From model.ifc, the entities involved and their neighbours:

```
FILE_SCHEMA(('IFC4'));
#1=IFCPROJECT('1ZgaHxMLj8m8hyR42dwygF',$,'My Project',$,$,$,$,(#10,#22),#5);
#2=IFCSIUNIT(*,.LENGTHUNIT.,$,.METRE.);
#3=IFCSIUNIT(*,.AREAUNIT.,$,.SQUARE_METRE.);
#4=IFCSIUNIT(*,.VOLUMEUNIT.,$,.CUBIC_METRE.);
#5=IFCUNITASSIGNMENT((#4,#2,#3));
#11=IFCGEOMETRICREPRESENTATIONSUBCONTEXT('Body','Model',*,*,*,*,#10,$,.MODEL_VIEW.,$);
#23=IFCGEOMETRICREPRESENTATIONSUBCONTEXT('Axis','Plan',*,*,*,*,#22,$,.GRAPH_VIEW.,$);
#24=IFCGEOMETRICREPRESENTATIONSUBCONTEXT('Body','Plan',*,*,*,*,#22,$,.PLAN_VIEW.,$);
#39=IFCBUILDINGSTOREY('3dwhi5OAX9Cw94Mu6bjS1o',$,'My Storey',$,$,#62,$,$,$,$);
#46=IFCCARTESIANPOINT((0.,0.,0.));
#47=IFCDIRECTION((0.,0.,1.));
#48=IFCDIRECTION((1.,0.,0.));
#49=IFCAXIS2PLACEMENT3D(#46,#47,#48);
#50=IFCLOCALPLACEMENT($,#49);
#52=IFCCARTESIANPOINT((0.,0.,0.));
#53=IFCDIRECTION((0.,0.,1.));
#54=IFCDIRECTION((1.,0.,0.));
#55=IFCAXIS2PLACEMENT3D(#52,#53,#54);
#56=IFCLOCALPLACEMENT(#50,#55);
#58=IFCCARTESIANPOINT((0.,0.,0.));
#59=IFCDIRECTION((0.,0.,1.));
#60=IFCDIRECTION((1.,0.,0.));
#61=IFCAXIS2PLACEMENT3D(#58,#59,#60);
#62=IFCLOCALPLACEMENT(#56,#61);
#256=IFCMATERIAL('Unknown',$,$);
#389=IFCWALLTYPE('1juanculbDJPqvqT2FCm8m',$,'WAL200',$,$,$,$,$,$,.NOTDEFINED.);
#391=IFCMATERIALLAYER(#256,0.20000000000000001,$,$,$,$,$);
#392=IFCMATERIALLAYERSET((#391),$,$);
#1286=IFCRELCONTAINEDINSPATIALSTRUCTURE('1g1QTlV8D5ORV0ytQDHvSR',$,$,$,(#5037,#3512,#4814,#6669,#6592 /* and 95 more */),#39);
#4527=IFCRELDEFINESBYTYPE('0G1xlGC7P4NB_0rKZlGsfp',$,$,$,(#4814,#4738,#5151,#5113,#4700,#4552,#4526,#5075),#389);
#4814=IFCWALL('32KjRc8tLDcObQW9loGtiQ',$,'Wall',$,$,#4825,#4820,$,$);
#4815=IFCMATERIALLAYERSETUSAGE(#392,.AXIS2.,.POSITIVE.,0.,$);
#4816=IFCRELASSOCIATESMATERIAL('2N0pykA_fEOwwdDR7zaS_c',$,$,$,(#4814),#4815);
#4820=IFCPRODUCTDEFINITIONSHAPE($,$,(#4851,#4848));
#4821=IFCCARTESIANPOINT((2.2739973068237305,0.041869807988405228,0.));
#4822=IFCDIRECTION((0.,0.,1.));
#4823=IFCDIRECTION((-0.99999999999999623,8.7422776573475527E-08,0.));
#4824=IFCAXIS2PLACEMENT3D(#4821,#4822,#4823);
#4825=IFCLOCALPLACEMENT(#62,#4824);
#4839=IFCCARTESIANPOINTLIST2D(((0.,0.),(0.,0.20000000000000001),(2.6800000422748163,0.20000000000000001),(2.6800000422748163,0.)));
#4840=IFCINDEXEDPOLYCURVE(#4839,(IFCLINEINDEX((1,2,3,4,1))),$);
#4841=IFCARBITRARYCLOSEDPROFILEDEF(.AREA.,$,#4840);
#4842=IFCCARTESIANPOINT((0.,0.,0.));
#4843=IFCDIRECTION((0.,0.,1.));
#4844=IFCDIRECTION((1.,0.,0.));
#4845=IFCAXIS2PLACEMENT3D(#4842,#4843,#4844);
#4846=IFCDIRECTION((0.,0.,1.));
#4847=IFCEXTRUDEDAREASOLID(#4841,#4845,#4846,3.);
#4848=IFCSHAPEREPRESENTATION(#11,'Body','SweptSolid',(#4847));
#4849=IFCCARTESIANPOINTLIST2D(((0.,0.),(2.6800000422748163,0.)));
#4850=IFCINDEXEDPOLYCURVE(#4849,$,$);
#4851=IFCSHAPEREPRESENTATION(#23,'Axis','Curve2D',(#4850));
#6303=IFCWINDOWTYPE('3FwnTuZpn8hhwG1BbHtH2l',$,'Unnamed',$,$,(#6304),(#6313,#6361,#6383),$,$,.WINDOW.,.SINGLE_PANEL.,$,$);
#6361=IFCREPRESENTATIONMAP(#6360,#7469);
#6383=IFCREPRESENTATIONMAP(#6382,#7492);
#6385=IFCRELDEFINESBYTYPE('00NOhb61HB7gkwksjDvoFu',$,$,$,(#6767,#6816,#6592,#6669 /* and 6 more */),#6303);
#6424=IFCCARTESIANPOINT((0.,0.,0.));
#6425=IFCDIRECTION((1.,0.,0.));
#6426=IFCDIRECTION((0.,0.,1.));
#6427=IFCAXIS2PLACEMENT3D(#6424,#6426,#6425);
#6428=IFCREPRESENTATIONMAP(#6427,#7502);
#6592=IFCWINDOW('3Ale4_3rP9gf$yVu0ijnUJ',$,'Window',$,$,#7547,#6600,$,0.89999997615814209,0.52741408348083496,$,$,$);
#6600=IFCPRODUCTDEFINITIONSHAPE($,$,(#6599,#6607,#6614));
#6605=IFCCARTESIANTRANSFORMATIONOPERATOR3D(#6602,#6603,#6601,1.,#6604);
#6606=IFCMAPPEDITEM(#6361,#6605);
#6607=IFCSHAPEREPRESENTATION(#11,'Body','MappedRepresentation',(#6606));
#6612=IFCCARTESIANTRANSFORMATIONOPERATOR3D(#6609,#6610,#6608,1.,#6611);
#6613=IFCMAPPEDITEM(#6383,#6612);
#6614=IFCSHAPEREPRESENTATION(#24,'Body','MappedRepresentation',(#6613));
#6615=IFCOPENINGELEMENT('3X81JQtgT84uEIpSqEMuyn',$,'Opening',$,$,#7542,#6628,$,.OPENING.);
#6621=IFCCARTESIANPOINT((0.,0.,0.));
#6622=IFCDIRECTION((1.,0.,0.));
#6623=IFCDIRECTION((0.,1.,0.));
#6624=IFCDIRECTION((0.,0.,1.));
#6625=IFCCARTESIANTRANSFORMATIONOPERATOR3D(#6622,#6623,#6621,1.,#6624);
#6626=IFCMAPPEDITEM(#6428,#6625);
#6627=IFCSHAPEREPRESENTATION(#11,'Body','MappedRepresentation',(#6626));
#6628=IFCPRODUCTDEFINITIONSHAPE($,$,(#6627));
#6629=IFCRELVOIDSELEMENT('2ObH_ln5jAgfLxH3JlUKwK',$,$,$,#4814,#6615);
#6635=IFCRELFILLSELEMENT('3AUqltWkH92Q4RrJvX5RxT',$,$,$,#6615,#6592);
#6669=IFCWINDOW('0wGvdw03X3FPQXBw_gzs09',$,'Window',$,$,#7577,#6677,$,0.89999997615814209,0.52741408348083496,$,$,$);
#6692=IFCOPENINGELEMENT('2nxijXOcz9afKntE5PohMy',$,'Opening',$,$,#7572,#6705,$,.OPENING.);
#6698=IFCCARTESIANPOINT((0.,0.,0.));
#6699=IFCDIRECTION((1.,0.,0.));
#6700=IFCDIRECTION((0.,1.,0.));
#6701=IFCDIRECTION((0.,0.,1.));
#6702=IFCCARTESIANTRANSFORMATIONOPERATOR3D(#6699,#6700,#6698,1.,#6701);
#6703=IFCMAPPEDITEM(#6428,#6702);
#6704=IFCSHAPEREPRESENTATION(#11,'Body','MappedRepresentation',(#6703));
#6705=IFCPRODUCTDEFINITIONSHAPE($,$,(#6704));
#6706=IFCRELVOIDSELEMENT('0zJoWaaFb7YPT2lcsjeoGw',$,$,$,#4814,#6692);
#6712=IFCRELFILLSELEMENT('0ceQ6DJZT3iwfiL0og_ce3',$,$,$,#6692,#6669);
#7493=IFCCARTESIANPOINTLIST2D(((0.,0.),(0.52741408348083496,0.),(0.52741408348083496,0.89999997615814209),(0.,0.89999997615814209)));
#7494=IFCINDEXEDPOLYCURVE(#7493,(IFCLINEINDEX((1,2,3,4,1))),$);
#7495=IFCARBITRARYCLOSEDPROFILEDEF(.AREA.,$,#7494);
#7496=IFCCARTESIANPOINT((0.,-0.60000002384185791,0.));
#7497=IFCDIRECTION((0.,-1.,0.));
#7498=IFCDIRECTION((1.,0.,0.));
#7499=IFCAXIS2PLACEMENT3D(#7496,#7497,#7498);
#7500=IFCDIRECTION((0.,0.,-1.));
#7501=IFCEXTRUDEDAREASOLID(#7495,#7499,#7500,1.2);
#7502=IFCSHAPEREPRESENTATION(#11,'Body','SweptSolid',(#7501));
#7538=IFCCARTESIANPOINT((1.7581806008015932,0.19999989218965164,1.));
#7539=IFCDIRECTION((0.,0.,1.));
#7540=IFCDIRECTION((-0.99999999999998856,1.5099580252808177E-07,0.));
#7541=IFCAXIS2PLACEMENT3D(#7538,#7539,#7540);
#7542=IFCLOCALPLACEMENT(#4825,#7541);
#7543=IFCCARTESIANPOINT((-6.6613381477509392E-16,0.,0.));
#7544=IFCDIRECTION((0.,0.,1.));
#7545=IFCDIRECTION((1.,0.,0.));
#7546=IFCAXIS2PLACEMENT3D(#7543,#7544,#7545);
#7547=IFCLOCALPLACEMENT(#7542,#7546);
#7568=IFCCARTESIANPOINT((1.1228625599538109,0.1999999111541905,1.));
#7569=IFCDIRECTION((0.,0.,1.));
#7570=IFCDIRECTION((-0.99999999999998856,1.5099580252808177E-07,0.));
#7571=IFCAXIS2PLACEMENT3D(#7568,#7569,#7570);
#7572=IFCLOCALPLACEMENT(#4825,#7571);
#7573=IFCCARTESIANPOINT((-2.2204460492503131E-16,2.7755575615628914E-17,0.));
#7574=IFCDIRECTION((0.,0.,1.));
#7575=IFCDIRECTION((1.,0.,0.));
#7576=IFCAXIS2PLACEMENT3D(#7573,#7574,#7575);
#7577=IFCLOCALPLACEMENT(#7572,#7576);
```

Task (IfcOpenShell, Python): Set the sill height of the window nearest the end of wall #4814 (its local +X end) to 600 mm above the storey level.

```python
import numpy as np
import ifcopenshell
import ifcopenshell.api.geometry
import ifcopenshell.geom
import ifcopenshell.util.element
import ifcopenshell.util.placement
import ifcopenshell.util.shape
import ifcopenshell.util.unit

model = ifcopenshell.open("model.ifc")
unit_scale = ifcopenshell.util.unit.calculate_unit_scale(model)

window = model.by_id(6592)
opening = window.FillsVoids[0].RelatingOpeningElement
storey = ifcopenshell.util.element.get_container(window, ifc_class="IfcBuildingStorey")
level = ifcopenshell.util.placement.get_local_placement(storey.ObjectPlacement)[2, 3]

# The opening's origin need not be at the sill, so measure its lowest point.
shape = ifcopenshell.geom.create_shape(ifcopenshell.geom.settings(), opening)
bottom = ifcopenshell.util.shape.get_shape_bottom_elevation(shape, shape.geometry) / unit_scale
dz = level + 0.6 / unit_scale - bottom

shift = np.array([0.0, 0.0, dz])
# The window is placed relative to its opening, so it follows when the opening moves.
matrix = ifcopenshell.util.placement.get_local_placement(opening.ObjectPlacement)
matrix[:3, 3] += shift
ifcopenshell.api.geometry.edit_object_placement(
    model, product=opening, matrix=matrix, is_si=False, should_transform_children=True
)

print(f"moved by {dz * unit_scale:+.3f} m")

model.write("model_v2.ifc")
```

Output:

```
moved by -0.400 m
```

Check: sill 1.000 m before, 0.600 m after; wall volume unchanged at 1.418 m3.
